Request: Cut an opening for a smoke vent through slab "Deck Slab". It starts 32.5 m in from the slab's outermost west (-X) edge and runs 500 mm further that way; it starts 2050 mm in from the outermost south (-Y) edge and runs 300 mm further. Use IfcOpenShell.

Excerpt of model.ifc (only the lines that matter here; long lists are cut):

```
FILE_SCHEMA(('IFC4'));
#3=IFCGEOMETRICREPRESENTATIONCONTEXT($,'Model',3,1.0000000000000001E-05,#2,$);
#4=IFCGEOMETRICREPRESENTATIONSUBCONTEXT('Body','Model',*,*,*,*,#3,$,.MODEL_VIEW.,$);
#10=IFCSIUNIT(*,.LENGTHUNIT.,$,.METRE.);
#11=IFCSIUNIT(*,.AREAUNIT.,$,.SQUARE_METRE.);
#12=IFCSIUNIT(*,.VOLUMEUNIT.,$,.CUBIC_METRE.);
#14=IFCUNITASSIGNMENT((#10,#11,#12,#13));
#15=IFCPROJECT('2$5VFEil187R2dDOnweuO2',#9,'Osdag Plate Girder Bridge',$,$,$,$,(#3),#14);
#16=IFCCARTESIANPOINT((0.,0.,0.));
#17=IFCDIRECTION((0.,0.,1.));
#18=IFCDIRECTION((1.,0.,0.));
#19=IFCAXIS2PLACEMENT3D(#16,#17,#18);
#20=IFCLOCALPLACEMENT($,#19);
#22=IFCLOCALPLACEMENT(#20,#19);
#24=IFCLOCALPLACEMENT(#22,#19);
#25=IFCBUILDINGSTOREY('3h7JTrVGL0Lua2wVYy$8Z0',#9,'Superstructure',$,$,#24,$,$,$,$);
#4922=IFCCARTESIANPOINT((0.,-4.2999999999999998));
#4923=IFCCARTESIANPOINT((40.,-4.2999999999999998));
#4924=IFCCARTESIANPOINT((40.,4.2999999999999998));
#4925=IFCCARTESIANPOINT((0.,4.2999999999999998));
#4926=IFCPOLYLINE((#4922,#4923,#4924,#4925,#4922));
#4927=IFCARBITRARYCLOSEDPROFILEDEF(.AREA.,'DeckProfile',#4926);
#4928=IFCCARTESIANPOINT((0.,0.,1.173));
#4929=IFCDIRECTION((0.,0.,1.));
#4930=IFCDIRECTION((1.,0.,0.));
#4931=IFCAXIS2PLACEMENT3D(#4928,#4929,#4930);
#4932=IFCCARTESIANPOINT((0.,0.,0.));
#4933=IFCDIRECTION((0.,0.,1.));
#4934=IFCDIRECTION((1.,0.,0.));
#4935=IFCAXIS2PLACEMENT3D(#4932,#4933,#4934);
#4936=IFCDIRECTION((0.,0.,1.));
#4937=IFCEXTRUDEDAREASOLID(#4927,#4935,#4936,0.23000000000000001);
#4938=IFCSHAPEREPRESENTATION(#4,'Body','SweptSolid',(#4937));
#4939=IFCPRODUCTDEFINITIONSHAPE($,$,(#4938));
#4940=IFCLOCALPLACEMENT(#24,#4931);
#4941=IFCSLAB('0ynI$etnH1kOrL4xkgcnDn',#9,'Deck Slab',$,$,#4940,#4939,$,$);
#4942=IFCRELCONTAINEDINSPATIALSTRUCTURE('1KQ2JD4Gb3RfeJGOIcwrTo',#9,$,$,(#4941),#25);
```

```python
import numpy as np
import ifcopenshell
import ifcopenshell.api.feature
import ifcopenshell.api.geometry
import ifcopenshell.api.root
import ifcopenshell.geom
import ifcopenshell.util.placement
import ifcopenshell.util.representation
import ifcopenshell.util.shape
import ifcopenshell.util.unit

model = ifcopenshell.open("model.ifc")
unit_scale = ifcopenshell.util.unit.calculate_unit_scale(model)
settings = ifcopenshell.geom.settings()


def volume(element):
    """Net volume in cubic metres, openings subtracted."""
    shape = ifcopenshell.geom.create_shape(settings, element)
    return ifcopenshell.util.shape.get_volume(shape.geometry)


slab = model.by_guid("0ynI$etnH1kOrL4xkgcnDn")
before = volume(slab)

# Extent in the slab's own axes, in metres. The edges named are its -X and -Y sides.
slab_shape = ifcopenshell.geom.create_shape(settings, slab)
vertices = ifcopenshell.util.shape.get_vertices(slab_shape.geometry)
x_min, y_min, bottom = vertices.min(axis=0)
top = vertices[:, 2].max()

opening = ifcopenshell.api.root.create_entity(model, ifc_class="IfcOpeningElement", name="Smoke vent opening", predefined_type="OPENING")
context = ifcopenshell.util.representation.get_context(model, "Model", "Body", "MODEL_VIEW")
width, depth = 0.5, 0.3
outline = [(0.0, 0.0), (width, 0.0), (width, depth), (0.0, depth), (0.0, 0.0)]
# Overshoot both faces by 50 mm so the cut is clean.
shape = ifcopenshell.api.geometry.add_slab_representation(
    model, context=context, depth=top - bottom + 0.1, polyline=outline
)
ifcopenshell.api.geometry.assign_representation(model, product=opening, representation=shape)

matrix = ifcopenshell.util.placement.get_local_placement(slab.ObjectPlacement)
matrix[:, 3] = matrix @ np.append(np.array([x_min + 32.5, y_min + 2.05, bottom - 0.05]) / unit_scale, 1.0)
ifcopenshell.api.geometry.edit_object_placement(model, product=opening, matrix=matrix, is_si=False)
ifcopenshell.api.feature.add_feature(model, feature=opening, element=slab)

after = volume(slab)

print(f"slab volume {before:.3f} -> {after:.3f} m3")

model.write("model_v2.ifc")
```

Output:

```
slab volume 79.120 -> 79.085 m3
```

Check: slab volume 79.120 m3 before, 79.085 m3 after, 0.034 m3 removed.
